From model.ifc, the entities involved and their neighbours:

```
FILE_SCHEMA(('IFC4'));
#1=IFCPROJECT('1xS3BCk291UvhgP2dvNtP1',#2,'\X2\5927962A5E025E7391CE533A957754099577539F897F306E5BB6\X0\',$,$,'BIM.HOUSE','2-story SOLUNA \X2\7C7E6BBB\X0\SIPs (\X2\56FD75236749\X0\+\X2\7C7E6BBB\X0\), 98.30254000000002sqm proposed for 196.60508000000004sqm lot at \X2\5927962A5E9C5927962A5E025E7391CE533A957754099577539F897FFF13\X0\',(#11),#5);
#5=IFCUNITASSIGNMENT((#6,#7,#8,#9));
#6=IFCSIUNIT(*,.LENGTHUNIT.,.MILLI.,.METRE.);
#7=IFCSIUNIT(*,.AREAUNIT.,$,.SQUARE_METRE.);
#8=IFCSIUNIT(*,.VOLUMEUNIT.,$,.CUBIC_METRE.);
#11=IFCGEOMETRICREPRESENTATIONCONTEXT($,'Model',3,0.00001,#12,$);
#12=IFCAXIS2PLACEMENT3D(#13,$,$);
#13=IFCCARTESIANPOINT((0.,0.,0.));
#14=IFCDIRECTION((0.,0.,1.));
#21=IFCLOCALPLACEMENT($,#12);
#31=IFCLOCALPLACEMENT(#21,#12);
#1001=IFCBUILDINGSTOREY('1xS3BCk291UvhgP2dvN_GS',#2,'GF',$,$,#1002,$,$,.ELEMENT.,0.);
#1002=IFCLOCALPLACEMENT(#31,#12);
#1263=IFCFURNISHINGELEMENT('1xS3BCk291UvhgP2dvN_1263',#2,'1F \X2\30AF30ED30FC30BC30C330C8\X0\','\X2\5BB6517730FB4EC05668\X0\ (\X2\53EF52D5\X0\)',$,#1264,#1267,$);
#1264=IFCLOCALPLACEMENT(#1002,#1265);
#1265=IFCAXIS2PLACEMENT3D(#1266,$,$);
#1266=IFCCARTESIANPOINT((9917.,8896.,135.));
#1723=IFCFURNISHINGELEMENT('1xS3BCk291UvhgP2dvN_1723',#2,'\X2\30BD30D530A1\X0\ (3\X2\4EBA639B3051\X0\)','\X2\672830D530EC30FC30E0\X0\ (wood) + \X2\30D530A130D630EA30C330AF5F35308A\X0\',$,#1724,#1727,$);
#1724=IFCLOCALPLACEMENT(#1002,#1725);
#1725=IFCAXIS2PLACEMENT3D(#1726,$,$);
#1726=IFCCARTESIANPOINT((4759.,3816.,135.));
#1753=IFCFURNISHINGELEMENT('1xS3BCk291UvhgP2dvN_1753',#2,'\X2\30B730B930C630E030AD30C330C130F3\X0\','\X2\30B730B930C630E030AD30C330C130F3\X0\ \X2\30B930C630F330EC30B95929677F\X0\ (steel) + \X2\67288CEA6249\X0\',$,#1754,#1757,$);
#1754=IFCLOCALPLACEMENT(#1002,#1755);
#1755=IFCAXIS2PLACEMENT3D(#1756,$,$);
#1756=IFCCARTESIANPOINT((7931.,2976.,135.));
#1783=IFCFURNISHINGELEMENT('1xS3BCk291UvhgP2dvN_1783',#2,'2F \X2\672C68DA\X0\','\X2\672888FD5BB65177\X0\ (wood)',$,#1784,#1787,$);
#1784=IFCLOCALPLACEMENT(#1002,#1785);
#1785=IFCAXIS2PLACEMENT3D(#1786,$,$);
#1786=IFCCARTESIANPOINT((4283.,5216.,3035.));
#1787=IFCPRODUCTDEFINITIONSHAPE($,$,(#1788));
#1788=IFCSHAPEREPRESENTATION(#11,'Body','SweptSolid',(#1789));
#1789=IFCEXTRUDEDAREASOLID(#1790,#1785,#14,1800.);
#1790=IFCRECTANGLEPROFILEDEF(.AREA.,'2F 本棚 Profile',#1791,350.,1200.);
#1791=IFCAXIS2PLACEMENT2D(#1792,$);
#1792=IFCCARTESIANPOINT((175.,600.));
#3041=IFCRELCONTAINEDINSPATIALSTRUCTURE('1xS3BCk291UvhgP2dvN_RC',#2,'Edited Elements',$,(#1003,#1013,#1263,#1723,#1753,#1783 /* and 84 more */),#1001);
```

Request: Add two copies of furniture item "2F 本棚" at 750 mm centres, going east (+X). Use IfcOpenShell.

```python
import numpy as np
import ifcopenshell
import ifcopenshell.api.geometry
import ifcopenshell.api.root
import ifcopenshell.util.element
import ifcopenshell.util.placement
import ifcopenshell.util.unit

model = ifcopenshell.open("model.ifc")
unit_scale = ifcopenshell.util.unit.calculate_unit_scale(model)


def reuse_history(source, copy):
    """copy_class also copies each property set's owner history, people and application; keep the originals."""
    for rel in copy.IsDefinedBy:
        if rel.is_a("IfcRelDefinesByProperties") and (history := rel.RelatingPropertyDefinition.OwnerHistory):
            rel.RelatingPropertyDefinition.OwnerHistory = source.OwnerHistory
            ifcopenshell.util.element.remove_deep2(model, history)


source = model.by_id(1783)
base = ifcopenshell.util.placement.get_local_placement(source.ObjectPlacement)
step = np.array([1.0, 0.0, 0.0]) * 0.75 / unit_scale

for i in range(1, 3):
    copy = ifcopenshell.api.root.copy_class(model, product=source)
    copy.Representation = ifcopenshell.util.element.copy_deep(
        model, source.Representation, exclude=["IfcGeometricRepresentationContext", "IfcRepresentationMap"]
    )
    reuse_history(source, copy)
    matrix = base.copy()
    matrix[:3, 3] += i * step
    print("added at", matrix[:3, 3].round(3) + 0.0)
    ifcopenshell.api.geometry.edit_object_placement(model, product=copy, matrix=matrix, is_si=False)

model.write("model_v2.ifc")
```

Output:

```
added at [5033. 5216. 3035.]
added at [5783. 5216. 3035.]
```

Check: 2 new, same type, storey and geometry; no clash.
